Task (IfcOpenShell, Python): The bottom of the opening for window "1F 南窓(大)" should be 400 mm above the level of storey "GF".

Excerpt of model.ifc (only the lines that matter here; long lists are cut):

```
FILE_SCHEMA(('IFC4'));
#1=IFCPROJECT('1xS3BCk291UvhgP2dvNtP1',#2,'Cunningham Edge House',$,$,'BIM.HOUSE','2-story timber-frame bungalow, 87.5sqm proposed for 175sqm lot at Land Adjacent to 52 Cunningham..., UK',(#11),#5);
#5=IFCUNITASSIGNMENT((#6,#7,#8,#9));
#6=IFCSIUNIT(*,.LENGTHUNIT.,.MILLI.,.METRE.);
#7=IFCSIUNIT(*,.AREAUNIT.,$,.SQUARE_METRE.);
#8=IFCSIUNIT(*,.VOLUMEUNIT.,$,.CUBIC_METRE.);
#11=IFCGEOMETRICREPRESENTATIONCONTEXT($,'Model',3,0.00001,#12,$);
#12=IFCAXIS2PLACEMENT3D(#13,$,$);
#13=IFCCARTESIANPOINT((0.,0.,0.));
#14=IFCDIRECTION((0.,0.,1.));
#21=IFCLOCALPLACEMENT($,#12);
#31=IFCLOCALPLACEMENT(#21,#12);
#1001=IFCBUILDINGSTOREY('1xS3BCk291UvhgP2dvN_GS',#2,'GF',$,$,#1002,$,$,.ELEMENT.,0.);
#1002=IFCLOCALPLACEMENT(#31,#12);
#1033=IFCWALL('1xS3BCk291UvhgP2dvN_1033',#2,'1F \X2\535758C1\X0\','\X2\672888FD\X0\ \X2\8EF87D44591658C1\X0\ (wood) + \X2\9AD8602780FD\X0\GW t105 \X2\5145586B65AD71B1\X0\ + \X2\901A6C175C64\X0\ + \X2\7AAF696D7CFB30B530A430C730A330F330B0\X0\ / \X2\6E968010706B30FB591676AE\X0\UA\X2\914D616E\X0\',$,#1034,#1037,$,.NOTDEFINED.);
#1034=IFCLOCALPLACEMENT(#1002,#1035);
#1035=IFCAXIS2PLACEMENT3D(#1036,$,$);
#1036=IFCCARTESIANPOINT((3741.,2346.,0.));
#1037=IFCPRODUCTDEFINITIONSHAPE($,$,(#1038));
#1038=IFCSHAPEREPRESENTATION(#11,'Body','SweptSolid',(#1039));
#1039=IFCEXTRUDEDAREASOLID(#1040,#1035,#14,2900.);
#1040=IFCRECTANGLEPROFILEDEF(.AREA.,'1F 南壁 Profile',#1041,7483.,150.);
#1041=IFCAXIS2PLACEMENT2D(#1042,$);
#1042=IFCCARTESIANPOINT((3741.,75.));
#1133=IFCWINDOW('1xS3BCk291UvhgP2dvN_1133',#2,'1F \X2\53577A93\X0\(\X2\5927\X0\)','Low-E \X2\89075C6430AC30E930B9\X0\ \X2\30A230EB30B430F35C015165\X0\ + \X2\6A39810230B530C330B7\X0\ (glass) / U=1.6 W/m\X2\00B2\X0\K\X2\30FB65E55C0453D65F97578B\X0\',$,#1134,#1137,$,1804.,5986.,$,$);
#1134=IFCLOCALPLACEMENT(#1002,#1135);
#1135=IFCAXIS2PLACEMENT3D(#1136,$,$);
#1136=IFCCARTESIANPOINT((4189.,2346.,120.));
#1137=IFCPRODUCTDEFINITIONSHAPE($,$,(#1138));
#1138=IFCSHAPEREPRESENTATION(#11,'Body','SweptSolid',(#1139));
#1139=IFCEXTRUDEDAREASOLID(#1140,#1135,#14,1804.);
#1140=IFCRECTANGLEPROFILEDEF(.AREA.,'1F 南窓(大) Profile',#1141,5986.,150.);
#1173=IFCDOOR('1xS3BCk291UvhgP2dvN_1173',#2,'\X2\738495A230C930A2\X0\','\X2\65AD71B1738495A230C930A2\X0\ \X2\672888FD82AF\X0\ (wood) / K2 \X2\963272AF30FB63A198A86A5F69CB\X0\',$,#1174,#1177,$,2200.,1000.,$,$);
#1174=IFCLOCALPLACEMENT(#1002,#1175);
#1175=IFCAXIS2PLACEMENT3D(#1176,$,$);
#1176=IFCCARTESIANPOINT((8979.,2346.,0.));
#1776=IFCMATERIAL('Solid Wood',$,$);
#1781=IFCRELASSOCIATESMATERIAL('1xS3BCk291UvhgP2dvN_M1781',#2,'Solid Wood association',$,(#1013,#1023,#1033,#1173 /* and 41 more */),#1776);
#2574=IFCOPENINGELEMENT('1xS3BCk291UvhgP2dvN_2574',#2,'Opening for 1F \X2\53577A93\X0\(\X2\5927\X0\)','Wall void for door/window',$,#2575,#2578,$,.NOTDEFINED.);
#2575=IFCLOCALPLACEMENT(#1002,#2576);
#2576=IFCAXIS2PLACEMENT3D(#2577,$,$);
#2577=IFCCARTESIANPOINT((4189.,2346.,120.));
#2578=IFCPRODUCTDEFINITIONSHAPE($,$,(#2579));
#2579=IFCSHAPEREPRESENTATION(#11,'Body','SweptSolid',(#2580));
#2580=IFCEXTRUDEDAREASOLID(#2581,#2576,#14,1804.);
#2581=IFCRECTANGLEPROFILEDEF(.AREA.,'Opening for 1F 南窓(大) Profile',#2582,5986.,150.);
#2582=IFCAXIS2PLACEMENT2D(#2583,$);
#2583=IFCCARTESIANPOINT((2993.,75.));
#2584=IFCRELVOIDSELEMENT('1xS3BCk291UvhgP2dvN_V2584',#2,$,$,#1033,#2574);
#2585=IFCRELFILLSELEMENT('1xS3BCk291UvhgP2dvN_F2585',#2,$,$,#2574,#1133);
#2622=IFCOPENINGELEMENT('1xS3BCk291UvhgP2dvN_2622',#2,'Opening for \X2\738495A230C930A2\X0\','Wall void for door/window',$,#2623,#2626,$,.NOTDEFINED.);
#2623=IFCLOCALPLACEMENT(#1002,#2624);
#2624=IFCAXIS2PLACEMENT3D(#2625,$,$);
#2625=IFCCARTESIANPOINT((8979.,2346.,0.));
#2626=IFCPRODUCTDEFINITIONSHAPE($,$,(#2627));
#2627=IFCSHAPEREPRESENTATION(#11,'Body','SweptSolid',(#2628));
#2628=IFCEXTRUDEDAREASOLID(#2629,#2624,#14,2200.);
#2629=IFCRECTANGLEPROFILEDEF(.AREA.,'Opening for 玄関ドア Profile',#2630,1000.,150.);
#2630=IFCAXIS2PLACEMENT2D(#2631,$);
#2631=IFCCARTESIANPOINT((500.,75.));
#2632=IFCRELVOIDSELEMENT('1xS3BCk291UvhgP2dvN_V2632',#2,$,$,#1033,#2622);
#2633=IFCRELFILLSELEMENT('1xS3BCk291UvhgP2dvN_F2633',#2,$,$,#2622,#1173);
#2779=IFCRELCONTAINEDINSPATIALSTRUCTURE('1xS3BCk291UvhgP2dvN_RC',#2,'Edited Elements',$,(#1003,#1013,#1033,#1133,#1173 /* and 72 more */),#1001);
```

```python
import numpy as np
import ifcopenshell
import ifcopenshell.api.geometry
import ifcopenshell.geom
import ifcopenshell.util.element
import ifcopenshell.util.placement
import ifcopenshell.util.shape
import ifcopenshell.util.unit

model = ifcopenshell.open("model.ifc")
unit_scale = ifcopenshell.util.unit.calculate_unit_scale(model)

window = model.by_guid("1xS3BCk291UvhgP2dvN_1133")
opening = window.FillsVoids[0].RelatingOpeningElement
storey = ifcopenshell.util.element.get_container(window, ifc_class="IfcBuildingStorey")
level = ifcopenshell.util.placement.get_local_placement(storey.ObjectPlacement)[2, 3]

# The opening's origin need not be at the sill, so measure its lowest point.
shape = ifcopenshell.geom.create_shape(ifcopenshell.geom.settings(), opening)
bottom = ifcopenshell.util.shape.get_shape_bottom_elevation(shape, shape.geometry) / unit_scale
dz = level + 0.4 / unit_scale - bottom

shift = np.array([0.0, 0.0, dz])
# The window is not placed relative to its opening, so move both.
for product in (opening, window):
    matrix = ifcopenshell.util.placement.get_local_placement(product.ObjectPlacement)
    matrix[:3, 3] += shift
    ifcopenshell.api.geometry.edit_object_placement(model, product=product, matrix=matrix, is_si=False)

print(f"moved by {dz * unit_scale:+.3f} m")

model.write("model-out.ifc")
```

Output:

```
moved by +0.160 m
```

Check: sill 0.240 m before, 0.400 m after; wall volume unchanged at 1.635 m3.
